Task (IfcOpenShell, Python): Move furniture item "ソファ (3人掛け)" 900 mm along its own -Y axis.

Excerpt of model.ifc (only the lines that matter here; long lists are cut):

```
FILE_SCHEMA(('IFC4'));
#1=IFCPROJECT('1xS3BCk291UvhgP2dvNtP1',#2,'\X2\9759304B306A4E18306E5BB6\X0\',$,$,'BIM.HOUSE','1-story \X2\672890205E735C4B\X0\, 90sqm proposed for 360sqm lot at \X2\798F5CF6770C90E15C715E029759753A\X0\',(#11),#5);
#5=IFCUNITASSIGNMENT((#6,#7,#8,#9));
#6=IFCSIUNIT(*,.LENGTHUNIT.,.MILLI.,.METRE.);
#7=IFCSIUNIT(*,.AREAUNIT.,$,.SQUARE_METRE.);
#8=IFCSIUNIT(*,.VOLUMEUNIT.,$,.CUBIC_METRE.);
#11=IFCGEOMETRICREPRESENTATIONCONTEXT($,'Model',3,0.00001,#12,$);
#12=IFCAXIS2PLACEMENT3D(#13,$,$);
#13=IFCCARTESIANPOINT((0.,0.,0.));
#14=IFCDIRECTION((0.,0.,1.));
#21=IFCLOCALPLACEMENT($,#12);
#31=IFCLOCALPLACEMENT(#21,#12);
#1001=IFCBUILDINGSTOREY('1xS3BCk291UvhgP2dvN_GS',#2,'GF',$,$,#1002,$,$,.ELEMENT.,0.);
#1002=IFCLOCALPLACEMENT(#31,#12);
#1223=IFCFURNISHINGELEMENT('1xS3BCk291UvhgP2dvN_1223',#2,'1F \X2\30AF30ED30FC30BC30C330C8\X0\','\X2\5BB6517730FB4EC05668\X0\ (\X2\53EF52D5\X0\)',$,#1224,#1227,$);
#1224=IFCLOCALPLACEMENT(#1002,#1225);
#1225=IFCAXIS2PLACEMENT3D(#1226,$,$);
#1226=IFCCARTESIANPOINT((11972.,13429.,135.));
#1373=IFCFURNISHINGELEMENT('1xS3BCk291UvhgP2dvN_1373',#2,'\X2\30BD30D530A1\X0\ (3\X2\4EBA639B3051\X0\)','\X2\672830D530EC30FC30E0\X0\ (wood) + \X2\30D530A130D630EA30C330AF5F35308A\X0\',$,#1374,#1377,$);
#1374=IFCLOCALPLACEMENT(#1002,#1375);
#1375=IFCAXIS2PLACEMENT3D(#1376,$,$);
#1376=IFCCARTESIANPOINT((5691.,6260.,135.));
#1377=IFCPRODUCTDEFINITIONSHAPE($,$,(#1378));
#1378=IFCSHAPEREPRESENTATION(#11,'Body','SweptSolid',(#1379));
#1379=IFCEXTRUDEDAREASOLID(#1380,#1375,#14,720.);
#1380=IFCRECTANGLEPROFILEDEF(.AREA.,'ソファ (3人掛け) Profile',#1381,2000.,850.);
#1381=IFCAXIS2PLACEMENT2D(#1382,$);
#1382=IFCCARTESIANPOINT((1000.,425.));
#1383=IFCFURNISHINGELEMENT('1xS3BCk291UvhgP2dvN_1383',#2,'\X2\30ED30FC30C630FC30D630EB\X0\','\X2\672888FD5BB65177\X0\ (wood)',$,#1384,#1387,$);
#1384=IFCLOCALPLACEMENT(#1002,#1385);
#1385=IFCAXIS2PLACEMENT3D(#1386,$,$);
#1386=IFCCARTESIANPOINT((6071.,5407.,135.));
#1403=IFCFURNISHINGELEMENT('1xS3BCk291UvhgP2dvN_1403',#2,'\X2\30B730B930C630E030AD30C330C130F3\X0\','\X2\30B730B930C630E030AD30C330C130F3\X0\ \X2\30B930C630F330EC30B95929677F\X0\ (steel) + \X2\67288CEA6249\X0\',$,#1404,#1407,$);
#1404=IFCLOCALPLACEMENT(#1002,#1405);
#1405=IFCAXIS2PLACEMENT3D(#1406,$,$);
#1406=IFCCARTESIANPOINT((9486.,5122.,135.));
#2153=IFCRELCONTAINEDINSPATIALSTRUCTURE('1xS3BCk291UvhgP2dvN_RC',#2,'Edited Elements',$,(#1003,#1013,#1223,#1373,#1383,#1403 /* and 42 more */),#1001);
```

```python
import ifcopenshell
import ifcopenshell.api.geometry
import ifcopenshell.util.placement
import ifcopenshell.util.unit

model = ifcopenshell.open("model.ifc")
unit_scale = ifcopenshell.util.unit.calculate_unit_scale(model)

item = model.by_guid("1xS3BCk291UvhgP2dvN_1373")
matrix = ifcopenshell.util.placement.get_local_placement(item.ObjectPlacement)
matrix[:3, 3] -= matrix[:3, 1] * 0.9 / unit_scale
ifcopenshell.api.geometry.edit_object_placement(model, product=item, matrix=matrix, is_si=False)

print(ifcopenshell.util.placement.get_local_placement(item.ObjectPlacement).round(3) + 0.0)

model.write("model_updated.ifc")
```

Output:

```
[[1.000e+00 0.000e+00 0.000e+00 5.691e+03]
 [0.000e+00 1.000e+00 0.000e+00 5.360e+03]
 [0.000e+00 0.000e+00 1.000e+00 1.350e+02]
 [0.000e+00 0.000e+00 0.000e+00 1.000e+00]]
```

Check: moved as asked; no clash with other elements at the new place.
